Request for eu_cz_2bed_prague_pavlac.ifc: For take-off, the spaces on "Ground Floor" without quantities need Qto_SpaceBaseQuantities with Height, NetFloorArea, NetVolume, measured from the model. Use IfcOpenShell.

First a look at what the model holds.

```python
import ifcopenshell
import ifcopenshell.util.element
import ifcopenshell.util.unit

model = ifcopenshell.open("eu_cz_2bed_prague_pavlac.ifc")
print(model.schema)
for unit_type in ("LENGTHUNIT", "AREAUNIT", "VOLUMEUNIT"):
    print(unit_type, ifcopenshell.util.unit.calculate_unit_scale(model, unit_type))
storey = next(s for s in model.by_type("IfcBuildingStorey") if s.Name == "Ground Floor")
spaces = [e for e in ifcopenshell.util.element.get_decomposition(storey) if e.is_a("IfcSpace")]
for e in sorted(spaces, key=lambda e: e.id()):
    print(e.id(), e.is_a(), e.Name, list(ifcopenshell.util.element.get_psets(e, qtos_only=True)), sep=" | ")
```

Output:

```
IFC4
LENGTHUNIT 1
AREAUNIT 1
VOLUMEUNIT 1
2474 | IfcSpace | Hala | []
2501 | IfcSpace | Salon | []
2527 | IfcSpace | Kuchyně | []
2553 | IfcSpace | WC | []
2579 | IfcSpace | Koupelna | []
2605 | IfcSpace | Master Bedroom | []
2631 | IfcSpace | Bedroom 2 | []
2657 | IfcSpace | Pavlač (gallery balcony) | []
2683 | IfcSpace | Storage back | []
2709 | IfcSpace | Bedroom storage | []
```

```python
import ifcopenshell
import ifcopenshell.api.pset
import ifcopenshell.geom
import ifcopenshell.util.element
import ifcopenshell.util.shape
import ifcopenshell.util.unit

model = ifcopenshell.open("eu_cz_2bed_prague_pavlac.ifc")
unit_scale = ifcopenshell.util.unit.calculate_unit_scale(model)
area_scale = ifcopenshell.util.unit.calculate_unit_scale(model, "AREAUNIT")
volume_scale = ifcopenshell.util.unit.calculate_unit_scale(model, "VOLUMEUNIT")
settings = ifcopenshell.geom.settings()

storey = next(s for s in model.by_type("IfcBuildingStorey") if s.Name == "Ground Floor")
spaces = [e for e in ifcopenshell.util.element.get_decomposition(storey) if e.is_a("IfcSpace")]

for e in sorted(spaces, key=lambda e: e.id()):
    if ifcopenshell.util.element.get_psets(e, qtos_only=True, should_inherit=False):
        continue
    # Geometry comes back in metres, in the element's own axes.
    shape = ifcopenshell.geom.create_shape(settings, e)
    values = {
        "Height": ifcopenshell.util.shape.get_z(shape.geometry) / unit_scale,
        "NetFloorArea": ifcopenshell.util.shape.get_footprint_area(shape.geometry) / area_scale,
        "NetVolume": ifcopenshell.util.shape.get_volume(shape.geometry) / volume_scale,
    }
    qto = ifcopenshell.api.pset.add_qto(model, product=e, name="Qto_SpaceBaseQuantities")
    ifcopenshell.api.pset.edit_qto(model, qto=qto, properties=values)
    print(e.id(), {k: round(v, 3) for k, v in values.items()})

model.write("eu_cz_2bed_prague_pavlac_edited.ifc")
```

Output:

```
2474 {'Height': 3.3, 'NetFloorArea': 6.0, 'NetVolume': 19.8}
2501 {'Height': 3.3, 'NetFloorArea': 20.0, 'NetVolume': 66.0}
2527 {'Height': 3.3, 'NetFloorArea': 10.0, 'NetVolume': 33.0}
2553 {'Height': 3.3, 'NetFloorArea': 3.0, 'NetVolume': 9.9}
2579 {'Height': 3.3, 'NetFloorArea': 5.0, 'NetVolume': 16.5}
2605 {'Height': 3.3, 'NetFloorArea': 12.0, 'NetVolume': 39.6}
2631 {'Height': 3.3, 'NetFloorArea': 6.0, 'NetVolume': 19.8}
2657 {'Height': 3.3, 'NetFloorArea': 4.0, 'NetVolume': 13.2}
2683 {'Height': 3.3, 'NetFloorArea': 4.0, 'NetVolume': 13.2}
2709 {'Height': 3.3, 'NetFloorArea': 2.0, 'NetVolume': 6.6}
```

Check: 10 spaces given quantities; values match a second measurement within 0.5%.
